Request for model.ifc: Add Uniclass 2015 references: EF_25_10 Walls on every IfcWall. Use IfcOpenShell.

First a look at what the model holds.

```python
import ifcopenshell

model = ifcopenshell.open("model.ifc")
print(model.schema)
print("classifications:", [c.Name for c in model.by_type("IfcClassification")])
for ifc_class in ("IfcDoor", "IfcRoof", "IfcStair", "IfcWall", "IfcWindow"):
    print(ifc_class, len(model.by_type(ifc_class)))
```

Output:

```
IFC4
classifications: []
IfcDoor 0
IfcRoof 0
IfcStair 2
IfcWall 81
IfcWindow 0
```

```python
import ifcopenshell
import ifcopenshell.api.classification

model = ifcopenshell.open("model.ifc")

system = ifcopenshell.api.classification.add_classification(model, classification="Uniclass 2015")

codes = {
    "IfcWall": ("EF_25_10", "Walls"),
}
for ifc_class, (code, name) in codes.items():
    products = model.by_type(ifc_class)
    ifcopenshell.api.classification.add_reference(
        model, products=products, classification=system, identification=code, name=name
    )
    print(code, len(products))

model.write("model-out.ifc")
```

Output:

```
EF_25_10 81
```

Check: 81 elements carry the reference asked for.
